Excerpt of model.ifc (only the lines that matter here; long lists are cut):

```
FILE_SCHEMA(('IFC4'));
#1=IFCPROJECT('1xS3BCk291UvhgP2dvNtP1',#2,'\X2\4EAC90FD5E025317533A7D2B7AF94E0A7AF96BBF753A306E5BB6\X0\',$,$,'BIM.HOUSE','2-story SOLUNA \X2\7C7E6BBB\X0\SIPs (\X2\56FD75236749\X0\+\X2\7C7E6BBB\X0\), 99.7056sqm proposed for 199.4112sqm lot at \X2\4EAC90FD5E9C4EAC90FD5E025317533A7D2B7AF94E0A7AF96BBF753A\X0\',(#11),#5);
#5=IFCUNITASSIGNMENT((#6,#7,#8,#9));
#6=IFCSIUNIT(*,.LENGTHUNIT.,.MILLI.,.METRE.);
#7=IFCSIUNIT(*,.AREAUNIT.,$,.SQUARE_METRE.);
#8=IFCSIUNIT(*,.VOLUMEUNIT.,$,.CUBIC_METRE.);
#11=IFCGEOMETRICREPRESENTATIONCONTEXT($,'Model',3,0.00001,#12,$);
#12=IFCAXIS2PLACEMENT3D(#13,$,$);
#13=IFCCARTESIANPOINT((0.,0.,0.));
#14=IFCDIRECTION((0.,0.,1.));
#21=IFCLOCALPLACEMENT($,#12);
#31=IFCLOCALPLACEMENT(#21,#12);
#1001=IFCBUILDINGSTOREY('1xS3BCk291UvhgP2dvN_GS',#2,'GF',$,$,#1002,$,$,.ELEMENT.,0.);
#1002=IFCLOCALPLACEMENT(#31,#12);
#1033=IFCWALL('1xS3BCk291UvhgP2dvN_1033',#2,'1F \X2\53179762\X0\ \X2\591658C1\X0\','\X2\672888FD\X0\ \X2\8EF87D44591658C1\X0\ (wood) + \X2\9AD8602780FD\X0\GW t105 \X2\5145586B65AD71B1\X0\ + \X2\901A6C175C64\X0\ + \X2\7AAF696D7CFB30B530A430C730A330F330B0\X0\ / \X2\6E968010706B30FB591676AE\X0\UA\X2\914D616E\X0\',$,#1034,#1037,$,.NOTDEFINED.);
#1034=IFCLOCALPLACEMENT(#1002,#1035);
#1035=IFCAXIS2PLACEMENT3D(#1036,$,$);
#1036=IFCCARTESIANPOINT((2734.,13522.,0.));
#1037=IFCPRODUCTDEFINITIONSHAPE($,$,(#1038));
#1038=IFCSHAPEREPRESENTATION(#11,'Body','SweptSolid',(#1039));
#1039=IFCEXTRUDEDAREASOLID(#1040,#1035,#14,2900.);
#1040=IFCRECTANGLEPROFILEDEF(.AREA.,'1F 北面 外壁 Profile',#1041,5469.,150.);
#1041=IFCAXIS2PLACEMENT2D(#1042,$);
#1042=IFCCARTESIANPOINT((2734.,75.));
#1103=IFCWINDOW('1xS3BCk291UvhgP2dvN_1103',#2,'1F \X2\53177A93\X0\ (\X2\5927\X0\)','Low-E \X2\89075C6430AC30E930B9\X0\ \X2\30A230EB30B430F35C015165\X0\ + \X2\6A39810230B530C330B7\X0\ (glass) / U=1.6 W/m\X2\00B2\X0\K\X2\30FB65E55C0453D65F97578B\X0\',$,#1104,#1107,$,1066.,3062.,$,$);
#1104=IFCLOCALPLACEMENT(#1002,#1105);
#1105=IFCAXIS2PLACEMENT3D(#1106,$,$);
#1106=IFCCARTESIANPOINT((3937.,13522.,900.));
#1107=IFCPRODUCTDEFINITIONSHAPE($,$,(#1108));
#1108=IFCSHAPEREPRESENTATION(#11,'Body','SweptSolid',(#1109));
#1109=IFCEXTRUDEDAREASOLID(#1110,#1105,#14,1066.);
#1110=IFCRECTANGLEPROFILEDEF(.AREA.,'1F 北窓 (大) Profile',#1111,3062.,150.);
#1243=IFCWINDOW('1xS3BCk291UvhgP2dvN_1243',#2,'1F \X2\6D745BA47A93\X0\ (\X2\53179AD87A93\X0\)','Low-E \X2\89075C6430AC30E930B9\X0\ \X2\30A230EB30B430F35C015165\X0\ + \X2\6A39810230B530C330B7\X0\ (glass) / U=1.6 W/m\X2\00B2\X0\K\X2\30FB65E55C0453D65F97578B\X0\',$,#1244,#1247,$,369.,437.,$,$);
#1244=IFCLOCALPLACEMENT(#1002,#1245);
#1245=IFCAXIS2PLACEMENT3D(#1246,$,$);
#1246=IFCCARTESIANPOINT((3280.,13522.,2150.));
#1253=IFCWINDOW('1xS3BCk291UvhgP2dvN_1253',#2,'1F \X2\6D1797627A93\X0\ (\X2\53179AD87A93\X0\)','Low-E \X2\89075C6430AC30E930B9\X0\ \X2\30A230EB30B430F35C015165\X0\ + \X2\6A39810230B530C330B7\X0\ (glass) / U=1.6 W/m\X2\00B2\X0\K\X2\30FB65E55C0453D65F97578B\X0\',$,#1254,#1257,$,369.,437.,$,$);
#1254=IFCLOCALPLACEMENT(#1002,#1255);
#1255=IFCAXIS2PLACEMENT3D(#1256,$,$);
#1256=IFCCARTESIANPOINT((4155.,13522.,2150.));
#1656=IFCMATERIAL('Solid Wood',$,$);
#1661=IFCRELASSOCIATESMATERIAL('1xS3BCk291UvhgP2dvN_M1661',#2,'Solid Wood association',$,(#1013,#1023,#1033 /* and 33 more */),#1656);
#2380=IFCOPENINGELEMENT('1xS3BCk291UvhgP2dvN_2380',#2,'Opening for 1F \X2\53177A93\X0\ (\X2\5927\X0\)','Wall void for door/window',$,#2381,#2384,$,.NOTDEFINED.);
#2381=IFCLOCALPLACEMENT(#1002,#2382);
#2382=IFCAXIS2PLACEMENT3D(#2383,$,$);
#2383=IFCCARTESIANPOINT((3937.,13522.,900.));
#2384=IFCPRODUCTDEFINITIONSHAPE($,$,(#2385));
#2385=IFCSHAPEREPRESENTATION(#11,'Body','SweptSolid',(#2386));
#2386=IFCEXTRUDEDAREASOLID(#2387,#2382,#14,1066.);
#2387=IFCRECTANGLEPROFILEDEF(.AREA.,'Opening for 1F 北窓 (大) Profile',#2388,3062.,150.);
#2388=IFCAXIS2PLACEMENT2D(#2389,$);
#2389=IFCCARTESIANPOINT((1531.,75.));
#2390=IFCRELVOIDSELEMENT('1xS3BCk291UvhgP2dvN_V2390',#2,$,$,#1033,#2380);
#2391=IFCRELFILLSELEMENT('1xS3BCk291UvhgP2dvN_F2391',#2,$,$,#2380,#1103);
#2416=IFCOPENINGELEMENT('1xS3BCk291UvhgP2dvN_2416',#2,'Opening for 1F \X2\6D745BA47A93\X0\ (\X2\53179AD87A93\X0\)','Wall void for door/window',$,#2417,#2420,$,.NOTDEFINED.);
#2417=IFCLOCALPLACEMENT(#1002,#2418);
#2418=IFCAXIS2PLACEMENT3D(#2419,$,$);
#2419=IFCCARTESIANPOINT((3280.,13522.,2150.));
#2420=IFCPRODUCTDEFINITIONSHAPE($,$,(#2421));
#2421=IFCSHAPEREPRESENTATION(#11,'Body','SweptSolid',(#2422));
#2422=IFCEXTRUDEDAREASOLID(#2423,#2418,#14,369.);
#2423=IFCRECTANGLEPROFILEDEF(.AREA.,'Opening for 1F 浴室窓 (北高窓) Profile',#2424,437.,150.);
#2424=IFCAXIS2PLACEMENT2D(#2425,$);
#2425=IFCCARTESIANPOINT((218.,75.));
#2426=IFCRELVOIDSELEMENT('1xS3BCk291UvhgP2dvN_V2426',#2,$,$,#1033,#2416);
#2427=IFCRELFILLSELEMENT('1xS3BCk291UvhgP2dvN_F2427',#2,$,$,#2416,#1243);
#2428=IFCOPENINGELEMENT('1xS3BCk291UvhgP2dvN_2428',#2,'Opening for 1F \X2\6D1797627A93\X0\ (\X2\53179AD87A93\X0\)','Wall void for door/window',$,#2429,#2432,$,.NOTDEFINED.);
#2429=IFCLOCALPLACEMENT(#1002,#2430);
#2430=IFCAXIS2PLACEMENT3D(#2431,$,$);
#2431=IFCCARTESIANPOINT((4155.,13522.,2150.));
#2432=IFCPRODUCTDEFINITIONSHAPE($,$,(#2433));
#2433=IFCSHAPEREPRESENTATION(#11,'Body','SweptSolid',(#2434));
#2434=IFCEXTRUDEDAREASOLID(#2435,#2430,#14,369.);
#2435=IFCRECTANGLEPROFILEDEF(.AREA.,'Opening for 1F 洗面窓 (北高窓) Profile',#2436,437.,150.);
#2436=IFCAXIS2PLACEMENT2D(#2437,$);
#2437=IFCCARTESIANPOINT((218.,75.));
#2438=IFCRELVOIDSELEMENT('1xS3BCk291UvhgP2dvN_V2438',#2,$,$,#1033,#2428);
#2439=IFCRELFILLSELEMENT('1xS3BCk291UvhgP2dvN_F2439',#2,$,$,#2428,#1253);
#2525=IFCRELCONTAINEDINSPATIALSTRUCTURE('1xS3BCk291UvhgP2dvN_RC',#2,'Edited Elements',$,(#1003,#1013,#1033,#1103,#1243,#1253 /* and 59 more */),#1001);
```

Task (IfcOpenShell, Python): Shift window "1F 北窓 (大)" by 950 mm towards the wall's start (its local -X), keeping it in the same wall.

```python
import ifcopenshell
import ifcopenshell.api.geometry
import ifcopenshell.util.placement
import ifcopenshell.util.unit

model = ifcopenshell.open("model.ifc")
unit_scale = ifcopenshell.util.unit.calculate_unit_scale(model)

window = model.by_id(1103)
opening = window.FillsVoids[0].RelatingOpeningElement
wall = opening.VoidsElements[0].RelatingBuildingElement

wall_matrix = ifcopenshell.util.placement.get_local_placement(wall.ObjectPlacement)
shift = wall_matrix[:3, 0] * -0.95 / unit_scale
before = ifcopenshell.util.placement.get_local_placement(window.ObjectPlacement)[:3, 3].copy()

# The window is not placed relative to its opening, so move both.
for product in (opening, window):
    matrix = ifcopenshell.util.placement.get_local_placement(product.ObjectPlacement)
    matrix[:3, 3] += shift
    ifcopenshell.api.geometry.edit_object_placement(model, product=product, matrix=matrix, is_si=False)

after = ifcopenshell.util.placement.get_local_placement(window.ObjectPlacement)[:3, 3]
print("window moved by", (after - before).round(3) + 0.0)

model.write("model_updated.ifc")
```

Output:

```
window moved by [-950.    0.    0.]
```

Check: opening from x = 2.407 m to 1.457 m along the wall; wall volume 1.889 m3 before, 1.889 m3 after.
